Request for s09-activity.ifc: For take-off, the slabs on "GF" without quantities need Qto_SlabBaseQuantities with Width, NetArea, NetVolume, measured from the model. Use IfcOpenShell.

First a look at what the model holds.

```python
import ifcopenshell
import ifcopenshell.util.element
import ifcopenshell.util.unit

model = ifcopenshell.open("s09-activity.ifc")
print(model.schema)
for unit_type in ("LENGTHUNIT", "AREAUNIT", "VOLUMEUNIT"):
    print(unit_type, ifcopenshell.util.unit.calculate_unit_scale(model, unit_type))
storey = next(s for s in model.by_type("IfcBuildingStorey") if s.Name == "GF")
slabs = [e for e in ifcopenshell.util.element.get_decomposition(storey) if e.is_a("IfcSlab")]
for e in sorted(slabs, key=lambda e: e.id()):
    print(e.id(), e.is_a(), e.Name, list(ifcopenshell.util.element.get_psets(e, qtos_only=True)), sep=" | ")
```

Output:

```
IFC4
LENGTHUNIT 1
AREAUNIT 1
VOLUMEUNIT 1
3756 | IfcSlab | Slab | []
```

```python
import ifcopenshell
import ifcopenshell.api.pset
import ifcopenshell.geom
import ifcopenshell.util.element
import ifcopenshell.util.shape
import ifcopenshell.util.unit

model = ifcopenshell.open("s09-activity.ifc")
unit_scale = ifcopenshell.util.unit.calculate_unit_scale(model)
area_scale = ifcopenshell.util.unit.calculate_unit_scale(model, "AREAUNIT")
volume_scale = ifcopenshell.util.unit.calculate_unit_scale(model, "VOLUMEUNIT")
settings = ifcopenshell.geom.settings()

storey = next(s for s in model.by_type("IfcBuildingStorey") if s.Name == "GF")
slabs = [e for e in ifcopenshell.util.element.get_decomposition(storey) if e.is_a("IfcSlab")]

for e in sorted(slabs, key=lambda e: e.id()):
    if ifcopenshell.util.element.get_psets(e, qtos_only=True, should_inherit=False):
        continue
    # Geometry comes back in metres, in the element's own axes.
    shape = ifcopenshell.geom.create_shape(settings, e)
    values = {
        "Width": ifcopenshell.util.shape.get_z(shape.geometry) / unit_scale,
        "NetArea": ifcopenshell.util.shape.get_footprint_area(shape.geometry) / area_scale,
        "NetVolume": ifcopenshell.util.shape.get_volume(shape.geometry) / volume_scale,
    }
    qto = ifcopenshell.api.pset.add_qto(model, product=e, name="Qto_SlabBaseQuantities")
    ifcopenshell.api.pset.edit_qto(model, qto=qto, properties=values)
    print(e.id(), {k: round(v, 3) for k, v in values.items()})

model.write("s09-activity_v2.ifc")
```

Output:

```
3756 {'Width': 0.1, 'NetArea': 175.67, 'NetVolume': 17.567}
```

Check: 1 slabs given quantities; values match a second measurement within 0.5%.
